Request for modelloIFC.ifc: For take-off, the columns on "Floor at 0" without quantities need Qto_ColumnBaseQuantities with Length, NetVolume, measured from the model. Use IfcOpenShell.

First a look at what the model holds.

```python
import ifcopenshell
import ifcopenshell.util.element
import ifcopenshell.util.unit

model = ifcopenshell.open("modelloIFC.ifc")
print(model.schema)
for unit_type in ("LENGTHUNIT", "AREAUNIT", "VOLUMEUNIT"):
    print(unit_type, ifcopenshell.util.unit.calculate_unit_scale(model, unit_type))
storey = next(s for s in model.by_type("IfcBuildingStorey") if s.Name == "Floor at 0")
columns = [e for e in ifcopenshell.util.element.get_decomposition(storey) if e.is_a("IfcColumn")]
for e in sorted(columns, key=lambda e: e.id()):
    print(e.id(), e.is_a(), e.Name, list(ifcopenshell.util.element.get_psets(e, qtos_only=True)), sep=" | ")
```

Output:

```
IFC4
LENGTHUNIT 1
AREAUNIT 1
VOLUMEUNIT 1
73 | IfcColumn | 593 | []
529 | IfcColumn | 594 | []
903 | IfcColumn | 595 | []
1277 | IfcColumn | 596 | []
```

```python
import ifcopenshell
import ifcopenshell.api.pset
import ifcopenshell.geom
import ifcopenshell.util.element
import ifcopenshell.util.shape
import ifcopenshell.util.unit

model = ifcopenshell.open("modelloIFC.ifc")
unit_scale = ifcopenshell.util.unit.calculate_unit_scale(model)
volume_scale = ifcopenshell.util.unit.calculate_unit_scale(model, "VOLUMEUNIT")
settings = ifcopenshell.geom.settings()

storey = next(s for s in model.by_type("IfcBuildingStorey") if s.Name == "Floor at 0")
columns = [e for e in ifcopenshell.util.element.get_decomposition(storey) if e.is_a("IfcColumn")]

for e in sorted(columns, key=lambda e: e.id()):
    if ifcopenshell.util.element.get_psets(e, qtos_only=True, should_inherit=False):
        continue
    # Geometry comes back in metres, in the element's own axes.
    shape = ifcopenshell.geom.create_shape(settings, e)
    values = {
        "Length": ifcopenshell.util.shape.get_z(shape.geometry) / unit_scale,
        "NetVolume": ifcopenshell.util.shape.get_volume(shape.geometry) / volume_scale,
    }
    qto = ifcopenshell.api.pset.add_qto(model, product=e, name="Qto_ColumnBaseQuantities")
    ifcopenshell.api.pset.edit_qto(model, qto=qto, properties=values)
    print(e.id(), {k: round(v, 3) for k, v in values.items()})

model.write("modelloIFC_rev.ifc")
```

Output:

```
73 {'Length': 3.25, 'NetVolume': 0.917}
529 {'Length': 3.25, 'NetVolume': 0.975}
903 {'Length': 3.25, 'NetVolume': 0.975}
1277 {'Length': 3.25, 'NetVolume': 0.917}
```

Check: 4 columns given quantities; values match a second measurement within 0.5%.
